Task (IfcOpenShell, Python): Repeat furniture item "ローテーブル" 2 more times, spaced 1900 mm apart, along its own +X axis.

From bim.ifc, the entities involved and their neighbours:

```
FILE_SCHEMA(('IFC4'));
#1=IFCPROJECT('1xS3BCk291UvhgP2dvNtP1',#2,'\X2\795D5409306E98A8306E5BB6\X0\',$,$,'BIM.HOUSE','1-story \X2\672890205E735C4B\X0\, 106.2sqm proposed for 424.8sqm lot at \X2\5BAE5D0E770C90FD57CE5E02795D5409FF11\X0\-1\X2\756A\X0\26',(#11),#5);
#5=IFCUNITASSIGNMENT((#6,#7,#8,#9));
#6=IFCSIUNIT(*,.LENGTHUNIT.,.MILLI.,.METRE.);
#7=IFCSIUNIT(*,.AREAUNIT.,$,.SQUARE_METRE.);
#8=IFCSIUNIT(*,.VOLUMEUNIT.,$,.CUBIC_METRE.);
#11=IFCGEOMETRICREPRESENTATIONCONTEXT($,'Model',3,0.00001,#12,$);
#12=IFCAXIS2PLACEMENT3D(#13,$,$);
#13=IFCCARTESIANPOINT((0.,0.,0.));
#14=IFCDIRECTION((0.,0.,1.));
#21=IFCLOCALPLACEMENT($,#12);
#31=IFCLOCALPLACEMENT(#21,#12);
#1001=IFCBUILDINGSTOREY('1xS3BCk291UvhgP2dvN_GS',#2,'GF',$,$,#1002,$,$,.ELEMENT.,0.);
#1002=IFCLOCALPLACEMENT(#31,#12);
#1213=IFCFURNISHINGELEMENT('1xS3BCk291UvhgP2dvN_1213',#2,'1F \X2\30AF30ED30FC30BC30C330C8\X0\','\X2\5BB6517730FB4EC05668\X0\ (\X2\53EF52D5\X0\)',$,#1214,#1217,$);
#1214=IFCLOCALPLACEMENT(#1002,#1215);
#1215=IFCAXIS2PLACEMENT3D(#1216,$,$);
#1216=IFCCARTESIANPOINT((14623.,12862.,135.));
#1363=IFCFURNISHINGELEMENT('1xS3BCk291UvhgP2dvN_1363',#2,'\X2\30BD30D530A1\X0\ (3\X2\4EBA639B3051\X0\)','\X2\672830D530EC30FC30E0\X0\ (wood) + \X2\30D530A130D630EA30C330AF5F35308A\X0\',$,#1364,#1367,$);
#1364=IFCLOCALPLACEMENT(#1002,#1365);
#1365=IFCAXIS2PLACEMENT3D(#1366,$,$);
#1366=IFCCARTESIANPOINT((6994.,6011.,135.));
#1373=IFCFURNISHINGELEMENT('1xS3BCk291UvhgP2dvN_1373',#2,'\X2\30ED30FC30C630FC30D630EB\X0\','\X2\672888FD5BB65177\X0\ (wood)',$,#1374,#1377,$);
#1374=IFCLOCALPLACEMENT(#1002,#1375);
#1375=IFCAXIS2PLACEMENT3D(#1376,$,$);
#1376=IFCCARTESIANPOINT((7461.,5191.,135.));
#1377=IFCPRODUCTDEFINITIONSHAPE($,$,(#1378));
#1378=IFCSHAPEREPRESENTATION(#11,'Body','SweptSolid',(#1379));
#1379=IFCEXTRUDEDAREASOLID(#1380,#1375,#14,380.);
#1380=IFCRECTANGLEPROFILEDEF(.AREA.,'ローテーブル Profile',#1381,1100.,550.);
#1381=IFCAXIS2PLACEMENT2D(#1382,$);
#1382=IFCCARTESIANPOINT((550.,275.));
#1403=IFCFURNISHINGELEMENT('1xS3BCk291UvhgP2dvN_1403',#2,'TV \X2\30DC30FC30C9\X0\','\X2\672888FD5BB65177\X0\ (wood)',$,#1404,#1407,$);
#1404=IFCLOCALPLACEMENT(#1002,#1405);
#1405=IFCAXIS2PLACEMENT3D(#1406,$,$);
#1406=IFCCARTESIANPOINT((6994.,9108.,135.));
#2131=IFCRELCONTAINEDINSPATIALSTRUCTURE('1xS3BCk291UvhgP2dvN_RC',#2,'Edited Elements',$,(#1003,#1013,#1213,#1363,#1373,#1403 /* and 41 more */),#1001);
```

```python
import ifcopenshell
import ifcopenshell.api.geometry
import ifcopenshell.api.root
import ifcopenshell.util.element
import ifcopenshell.util.placement

model = ifcopenshell.open("bim.ifc")


def reuse_history(source, copy):
    """copy_class also copies each property set's owner history, people and application; keep the originals."""
    for rel in copy.IsDefinedBy:
        if rel.is_a("IfcRelDefinesByProperties") and (history := rel.RelatingPropertyDefinition.OwnerHistory):
            rel.RelatingPropertyDefinition.OwnerHistory = source.OwnerHistory
            ifcopenshell.util.element.remove_deep2(model, history)


source = model.by_guid("1xS3BCk291UvhgP2dvN_1373")
base = ifcopenshell.util.placement.get_local_placement(source.ObjectPlacement)
step = base[:3, 0] * 1900.0

for i in range(1, 3):
    copy = ifcopenshell.api.root.copy_class(model, product=source)
    copy.Representation = ifcopenshell.util.element.copy_deep(
        model, source.Representation, exclude=["IfcGeometricRepresentationContext", "IfcRepresentationMap"]
    )
    reuse_history(source, copy)
    matrix = base.copy()
    matrix[:3, 3] += i * step
    print("added at", matrix[:3, 3].round(3) + 0.0)
    ifcopenshell.api.geometry.edit_object_placement(model, product=copy, matrix=matrix, is_si=False)

model.write("bim_updated.ifc")
```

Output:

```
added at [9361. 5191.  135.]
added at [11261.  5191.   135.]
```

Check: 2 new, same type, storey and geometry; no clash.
